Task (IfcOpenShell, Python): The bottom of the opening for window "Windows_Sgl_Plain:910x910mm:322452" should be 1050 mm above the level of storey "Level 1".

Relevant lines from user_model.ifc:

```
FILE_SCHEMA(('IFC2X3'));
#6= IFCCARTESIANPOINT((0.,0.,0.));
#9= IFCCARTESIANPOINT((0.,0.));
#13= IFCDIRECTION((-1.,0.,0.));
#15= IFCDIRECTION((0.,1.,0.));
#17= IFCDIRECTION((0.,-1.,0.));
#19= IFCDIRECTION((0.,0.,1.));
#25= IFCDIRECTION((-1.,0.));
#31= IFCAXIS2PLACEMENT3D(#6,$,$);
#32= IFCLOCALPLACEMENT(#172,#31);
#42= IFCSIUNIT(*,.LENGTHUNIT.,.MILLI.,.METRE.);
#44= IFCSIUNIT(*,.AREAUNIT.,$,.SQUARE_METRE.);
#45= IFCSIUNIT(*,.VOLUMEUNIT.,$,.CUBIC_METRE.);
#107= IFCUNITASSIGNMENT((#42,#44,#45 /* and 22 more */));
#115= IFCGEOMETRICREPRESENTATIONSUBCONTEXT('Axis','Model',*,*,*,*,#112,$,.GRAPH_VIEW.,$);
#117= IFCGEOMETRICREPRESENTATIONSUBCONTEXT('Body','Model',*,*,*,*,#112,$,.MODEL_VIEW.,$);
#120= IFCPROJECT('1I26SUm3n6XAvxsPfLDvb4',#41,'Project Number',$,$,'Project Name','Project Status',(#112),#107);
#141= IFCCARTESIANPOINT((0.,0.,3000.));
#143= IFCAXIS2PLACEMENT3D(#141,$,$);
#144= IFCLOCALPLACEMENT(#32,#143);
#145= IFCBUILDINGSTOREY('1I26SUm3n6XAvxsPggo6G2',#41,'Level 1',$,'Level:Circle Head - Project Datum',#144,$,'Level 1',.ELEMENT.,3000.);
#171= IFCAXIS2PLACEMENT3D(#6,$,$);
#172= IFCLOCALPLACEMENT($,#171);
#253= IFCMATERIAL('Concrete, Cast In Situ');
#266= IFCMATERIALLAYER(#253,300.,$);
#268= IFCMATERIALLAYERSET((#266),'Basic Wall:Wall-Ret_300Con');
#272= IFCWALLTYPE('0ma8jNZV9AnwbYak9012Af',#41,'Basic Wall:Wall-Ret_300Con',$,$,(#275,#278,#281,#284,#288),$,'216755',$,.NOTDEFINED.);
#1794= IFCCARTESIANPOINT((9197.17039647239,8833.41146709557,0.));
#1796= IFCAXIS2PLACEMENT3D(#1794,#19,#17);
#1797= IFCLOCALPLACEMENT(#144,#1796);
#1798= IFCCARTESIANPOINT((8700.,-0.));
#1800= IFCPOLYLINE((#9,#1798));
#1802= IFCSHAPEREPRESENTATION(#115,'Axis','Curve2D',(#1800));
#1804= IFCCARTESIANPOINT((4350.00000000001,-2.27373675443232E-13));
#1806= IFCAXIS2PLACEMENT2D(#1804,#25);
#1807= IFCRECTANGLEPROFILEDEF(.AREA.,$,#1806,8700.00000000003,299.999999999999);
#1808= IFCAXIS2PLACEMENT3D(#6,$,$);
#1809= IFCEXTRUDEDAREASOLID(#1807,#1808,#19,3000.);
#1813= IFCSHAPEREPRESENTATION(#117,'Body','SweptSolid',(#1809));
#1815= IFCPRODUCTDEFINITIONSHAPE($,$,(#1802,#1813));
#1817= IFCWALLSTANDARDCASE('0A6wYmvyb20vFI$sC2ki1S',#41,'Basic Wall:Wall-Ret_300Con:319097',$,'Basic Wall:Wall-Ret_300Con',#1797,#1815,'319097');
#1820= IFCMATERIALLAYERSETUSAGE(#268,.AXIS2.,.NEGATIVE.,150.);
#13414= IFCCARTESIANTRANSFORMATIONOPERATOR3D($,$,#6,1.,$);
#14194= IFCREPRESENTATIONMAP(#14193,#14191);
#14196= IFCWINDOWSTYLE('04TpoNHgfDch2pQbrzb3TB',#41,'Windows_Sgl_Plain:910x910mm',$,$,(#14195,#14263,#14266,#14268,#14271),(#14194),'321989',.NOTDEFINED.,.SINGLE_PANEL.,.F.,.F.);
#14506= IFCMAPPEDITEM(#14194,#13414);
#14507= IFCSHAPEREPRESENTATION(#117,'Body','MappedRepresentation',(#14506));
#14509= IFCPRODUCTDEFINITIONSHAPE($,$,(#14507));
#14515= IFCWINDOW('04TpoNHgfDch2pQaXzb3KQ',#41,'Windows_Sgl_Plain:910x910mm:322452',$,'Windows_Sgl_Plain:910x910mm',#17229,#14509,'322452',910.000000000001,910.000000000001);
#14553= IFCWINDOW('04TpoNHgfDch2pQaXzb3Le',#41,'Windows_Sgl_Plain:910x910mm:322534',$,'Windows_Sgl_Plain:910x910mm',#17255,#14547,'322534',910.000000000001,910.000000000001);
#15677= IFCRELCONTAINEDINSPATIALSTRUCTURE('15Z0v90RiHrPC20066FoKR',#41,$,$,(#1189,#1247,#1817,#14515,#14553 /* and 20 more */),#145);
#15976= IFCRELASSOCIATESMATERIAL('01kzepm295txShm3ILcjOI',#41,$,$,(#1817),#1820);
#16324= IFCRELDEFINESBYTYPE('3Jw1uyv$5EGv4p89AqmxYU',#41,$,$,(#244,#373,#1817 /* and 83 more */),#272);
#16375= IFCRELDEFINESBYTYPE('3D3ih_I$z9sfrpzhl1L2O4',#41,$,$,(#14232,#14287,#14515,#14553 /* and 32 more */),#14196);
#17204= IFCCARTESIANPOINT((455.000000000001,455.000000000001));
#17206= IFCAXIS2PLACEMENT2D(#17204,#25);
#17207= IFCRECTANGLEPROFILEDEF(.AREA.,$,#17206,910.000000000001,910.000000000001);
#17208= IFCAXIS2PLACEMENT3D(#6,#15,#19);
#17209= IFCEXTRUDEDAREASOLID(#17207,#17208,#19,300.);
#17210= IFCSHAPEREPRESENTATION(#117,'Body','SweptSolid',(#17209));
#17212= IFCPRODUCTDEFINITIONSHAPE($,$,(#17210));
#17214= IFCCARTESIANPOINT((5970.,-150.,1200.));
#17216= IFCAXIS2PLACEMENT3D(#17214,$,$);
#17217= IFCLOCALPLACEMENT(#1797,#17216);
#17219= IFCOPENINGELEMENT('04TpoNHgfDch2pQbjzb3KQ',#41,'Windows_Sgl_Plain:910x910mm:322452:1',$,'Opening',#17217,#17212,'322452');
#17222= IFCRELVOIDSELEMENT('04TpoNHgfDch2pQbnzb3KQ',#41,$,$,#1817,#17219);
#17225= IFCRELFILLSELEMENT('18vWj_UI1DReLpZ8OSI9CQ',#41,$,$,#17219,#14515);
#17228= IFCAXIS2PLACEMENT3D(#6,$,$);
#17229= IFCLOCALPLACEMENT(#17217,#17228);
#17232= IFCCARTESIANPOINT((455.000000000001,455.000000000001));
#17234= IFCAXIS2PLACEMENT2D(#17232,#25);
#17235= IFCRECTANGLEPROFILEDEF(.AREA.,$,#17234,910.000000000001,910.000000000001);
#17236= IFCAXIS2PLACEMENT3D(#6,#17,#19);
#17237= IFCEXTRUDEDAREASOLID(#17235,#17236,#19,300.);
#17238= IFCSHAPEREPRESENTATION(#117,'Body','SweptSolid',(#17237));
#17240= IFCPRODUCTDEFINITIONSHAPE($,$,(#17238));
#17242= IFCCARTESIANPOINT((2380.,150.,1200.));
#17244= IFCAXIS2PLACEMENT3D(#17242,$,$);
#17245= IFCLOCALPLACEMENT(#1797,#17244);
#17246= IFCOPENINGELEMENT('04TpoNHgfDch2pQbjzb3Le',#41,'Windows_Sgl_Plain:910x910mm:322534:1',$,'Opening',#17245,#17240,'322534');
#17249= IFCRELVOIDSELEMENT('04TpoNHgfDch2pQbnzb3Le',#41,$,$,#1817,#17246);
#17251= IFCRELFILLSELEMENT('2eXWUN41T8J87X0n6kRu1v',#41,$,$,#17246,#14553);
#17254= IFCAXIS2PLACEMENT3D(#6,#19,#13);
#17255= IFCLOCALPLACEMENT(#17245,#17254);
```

```python
import numpy as np
import ifcopenshell
import ifcopenshell.api.geometry
import ifcopenshell.geom
import ifcopenshell.util.element
import ifcopenshell.util.placement
import ifcopenshell.util.shape
import ifcopenshell.util.unit

model = ifcopenshell.open("user_model.ifc")
unit_scale = ifcopenshell.util.unit.calculate_unit_scale(model)

window = model.by_id(14515)
opening = window.FillsVoids[0].RelatingOpeningElement
storey = ifcopenshell.util.element.get_container(window, ifc_class="IfcBuildingStorey")
level = ifcopenshell.util.placement.get_local_placement(storey.ObjectPlacement)[2, 3]

# The opening's origin need not be at the sill, so measure its lowest point.
shape = ifcopenshell.geom.create_shape(ifcopenshell.geom.settings(), opening)
bottom = ifcopenshell.util.shape.get_shape_bottom_elevation(shape, shape.geometry) / unit_scale
dz = level + 1.05 / unit_scale - bottom

shift = np.array([0.0, 0.0, dz])
# The window is placed relative to its opening, so it follows when the opening moves.
matrix = ifcopenshell.util.placement.get_local_placement(opening.ObjectPlacement)
matrix[:3, 3] += shift
ifcopenshell.api.geometry.edit_object_placement(
    model, product=opening, matrix=matrix, is_si=False, should_transform_children=True
)

print(f"moved by {dz * unit_scale:+.3f} m")

model.write("user_model-out.ifc")
```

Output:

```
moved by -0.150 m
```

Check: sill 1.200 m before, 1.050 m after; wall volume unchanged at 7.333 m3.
